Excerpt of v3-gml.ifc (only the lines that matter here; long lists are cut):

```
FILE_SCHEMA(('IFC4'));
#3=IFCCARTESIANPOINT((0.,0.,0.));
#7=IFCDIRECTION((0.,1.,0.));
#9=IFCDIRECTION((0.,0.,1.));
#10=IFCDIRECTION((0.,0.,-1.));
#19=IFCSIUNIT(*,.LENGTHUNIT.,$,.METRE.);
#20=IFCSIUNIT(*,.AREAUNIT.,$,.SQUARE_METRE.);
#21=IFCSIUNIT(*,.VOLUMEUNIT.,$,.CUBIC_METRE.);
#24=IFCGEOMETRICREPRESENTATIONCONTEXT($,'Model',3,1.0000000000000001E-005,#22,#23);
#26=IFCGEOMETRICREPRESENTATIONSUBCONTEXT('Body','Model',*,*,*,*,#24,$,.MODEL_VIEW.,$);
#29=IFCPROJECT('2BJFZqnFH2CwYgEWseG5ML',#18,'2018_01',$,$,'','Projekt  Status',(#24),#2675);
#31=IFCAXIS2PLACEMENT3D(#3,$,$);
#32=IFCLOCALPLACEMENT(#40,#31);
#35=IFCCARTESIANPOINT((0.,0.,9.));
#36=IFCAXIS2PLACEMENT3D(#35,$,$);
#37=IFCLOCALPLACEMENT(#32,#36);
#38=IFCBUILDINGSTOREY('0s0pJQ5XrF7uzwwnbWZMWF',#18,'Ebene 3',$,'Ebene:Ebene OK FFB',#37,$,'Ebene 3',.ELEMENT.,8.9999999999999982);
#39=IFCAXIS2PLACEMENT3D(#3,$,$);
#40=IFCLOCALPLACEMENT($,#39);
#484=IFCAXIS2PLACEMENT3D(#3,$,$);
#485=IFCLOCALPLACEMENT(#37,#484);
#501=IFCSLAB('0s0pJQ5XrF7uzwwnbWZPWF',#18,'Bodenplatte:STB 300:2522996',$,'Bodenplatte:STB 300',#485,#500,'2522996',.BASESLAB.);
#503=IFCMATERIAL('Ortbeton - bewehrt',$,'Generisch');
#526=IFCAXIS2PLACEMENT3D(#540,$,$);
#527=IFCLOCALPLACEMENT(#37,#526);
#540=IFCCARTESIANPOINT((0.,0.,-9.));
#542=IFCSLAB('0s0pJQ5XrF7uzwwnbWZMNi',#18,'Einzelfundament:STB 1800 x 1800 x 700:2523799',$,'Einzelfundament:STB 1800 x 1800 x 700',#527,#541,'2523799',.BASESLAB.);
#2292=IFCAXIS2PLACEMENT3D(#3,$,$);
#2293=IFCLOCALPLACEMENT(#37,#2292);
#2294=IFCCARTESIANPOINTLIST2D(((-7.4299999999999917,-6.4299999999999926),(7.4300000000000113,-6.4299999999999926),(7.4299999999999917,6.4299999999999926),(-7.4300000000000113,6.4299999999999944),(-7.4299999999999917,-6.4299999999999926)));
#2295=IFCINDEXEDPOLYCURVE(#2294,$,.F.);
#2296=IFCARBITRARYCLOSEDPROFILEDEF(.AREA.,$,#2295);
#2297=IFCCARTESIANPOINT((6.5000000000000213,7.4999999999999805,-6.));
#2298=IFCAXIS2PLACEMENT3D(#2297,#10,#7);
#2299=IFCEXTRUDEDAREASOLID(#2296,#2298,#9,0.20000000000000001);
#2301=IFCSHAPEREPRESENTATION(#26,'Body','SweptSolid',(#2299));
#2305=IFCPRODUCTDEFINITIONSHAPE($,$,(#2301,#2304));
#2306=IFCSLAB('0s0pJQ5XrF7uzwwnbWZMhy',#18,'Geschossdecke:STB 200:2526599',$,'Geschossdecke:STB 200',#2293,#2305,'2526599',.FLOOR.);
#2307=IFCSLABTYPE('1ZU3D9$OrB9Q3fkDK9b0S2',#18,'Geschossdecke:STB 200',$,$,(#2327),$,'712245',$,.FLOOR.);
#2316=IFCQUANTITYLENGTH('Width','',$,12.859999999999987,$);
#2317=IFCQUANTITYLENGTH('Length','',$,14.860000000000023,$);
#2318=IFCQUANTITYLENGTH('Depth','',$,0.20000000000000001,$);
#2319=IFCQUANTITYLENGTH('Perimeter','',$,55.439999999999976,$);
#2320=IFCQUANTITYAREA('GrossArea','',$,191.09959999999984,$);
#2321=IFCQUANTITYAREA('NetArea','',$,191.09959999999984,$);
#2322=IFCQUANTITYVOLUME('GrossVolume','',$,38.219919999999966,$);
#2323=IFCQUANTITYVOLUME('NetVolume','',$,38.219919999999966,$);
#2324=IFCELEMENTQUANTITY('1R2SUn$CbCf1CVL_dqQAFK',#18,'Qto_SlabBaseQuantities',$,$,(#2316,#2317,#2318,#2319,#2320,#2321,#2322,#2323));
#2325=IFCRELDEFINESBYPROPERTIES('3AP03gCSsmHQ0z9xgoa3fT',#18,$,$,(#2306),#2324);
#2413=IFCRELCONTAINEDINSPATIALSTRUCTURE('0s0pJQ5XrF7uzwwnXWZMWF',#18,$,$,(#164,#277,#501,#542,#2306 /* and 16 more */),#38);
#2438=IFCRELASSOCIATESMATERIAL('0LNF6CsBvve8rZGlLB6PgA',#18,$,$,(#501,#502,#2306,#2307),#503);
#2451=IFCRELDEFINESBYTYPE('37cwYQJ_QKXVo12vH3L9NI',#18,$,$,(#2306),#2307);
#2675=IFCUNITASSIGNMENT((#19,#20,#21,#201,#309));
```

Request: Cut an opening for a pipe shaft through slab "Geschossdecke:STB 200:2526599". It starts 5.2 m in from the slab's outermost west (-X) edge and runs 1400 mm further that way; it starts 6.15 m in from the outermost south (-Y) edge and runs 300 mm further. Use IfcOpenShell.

```python
import numpy as np
import ifcopenshell
import ifcopenshell.api.feature
import ifcopenshell.api.geometry
import ifcopenshell.api.pset
import ifcopenshell.api.root
import ifcopenshell.geom
import ifcopenshell.util.element
import ifcopenshell.util.placement
import ifcopenshell.util.representation
import ifcopenshell.util.shape
import ifcopenshell.util.unit

model = ifcopenshell.open("v3-gml.ifc")
unit_scale = ifcopenshell.util.unit.calculate_unit_scale(model)
area_scale = ifcopenshell.util.unit.calculate_unit_scale(model, "AREAUNIT")
volume_scale = ifcopenshell.util.unit.calculate_unit_scale(model, "VOLUMEUNIT")
settings = ifcopenshell.geom.settings()


def volume(element):
    """Net volume in cubic metres, openings subtracted."""
    shape = ifcopenshell.geom.create_shape(settings, element)
    return ifcopenshell.util.shape.get_volume(shape.geometry)


slab = model.by_guid("0s0pJQ5XrF7uzwwnbWZMhy")
before = volume(slab)

# Extent in the slab's own axes, in metres. The edges named are its -X and -Y sides.
slab_shape = ifcopenshell.geom.create_shape(settings, slab)
vertices = ifcopenshell.util.shape.get_vertices(slab_shape.geometry)
x_min, y_min, bottom = vertices.min(axis=0)
top = vertices[:, 2].max()

opening = ifcopenshell.api.root.create_entity(model, ifc_class="IfcOpeningElement", name="Pipe shaft opening", predefined_type="OPENING")
context = ifcopenshell.util.representation.get_context(model, "Model", "Body", "MODEL_VIEW")
width, depth = 1.4, 0.3
outline = [(0.0, 0.0), (width, 0.0), (width, depth), (0.0, depth), (0.0, 0.0)]
# Overshoot both faces by 50 mm so the cut is clean.
shape = ifcopenshell.api.geometry.add_slab_representation(
    model, context=context, depth=top - bottom + 0.1, polyline=outline
)
ifcopenshell.api.geometry.assign_representation(model, product=opening, representation=shape)

matrix = ifcopenshell.util.placement.get_local_placement(slab.ObjectPlacement)
matrix[:, 3] = matrix @ np.append(np.array([x_min + 5.2, y_min + 6.15, bottom - 0.05]) / unit_scale, 1.0)
ifcopenshell.api.geometry.edit_object_placement(model, product=opening, matrix=matrix, is_si=False)
ifcopenshell.api.feature.add_feature(model, feature=opening, element=slab)

after = volume(slab)

# Update the slab's stored quantities.
qto = model.by_id(ifcopenshell.util.element.get_pset(slab, "Qto_SlabBaseQuantities", should_inherit=False)["id"])
ifcopenshell.api.pset.edit_qto(model, qto=qto, properties={
    "NetArea": after / (top - bottom) / area_scale,
    "NetVolume": after / volume_scale,
})

print(f"slab volume {before:.3f} -> {after:.3f} m3")

model.write("v3-gml-out.ifc")
```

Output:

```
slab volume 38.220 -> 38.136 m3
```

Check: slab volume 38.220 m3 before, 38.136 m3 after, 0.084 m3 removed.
